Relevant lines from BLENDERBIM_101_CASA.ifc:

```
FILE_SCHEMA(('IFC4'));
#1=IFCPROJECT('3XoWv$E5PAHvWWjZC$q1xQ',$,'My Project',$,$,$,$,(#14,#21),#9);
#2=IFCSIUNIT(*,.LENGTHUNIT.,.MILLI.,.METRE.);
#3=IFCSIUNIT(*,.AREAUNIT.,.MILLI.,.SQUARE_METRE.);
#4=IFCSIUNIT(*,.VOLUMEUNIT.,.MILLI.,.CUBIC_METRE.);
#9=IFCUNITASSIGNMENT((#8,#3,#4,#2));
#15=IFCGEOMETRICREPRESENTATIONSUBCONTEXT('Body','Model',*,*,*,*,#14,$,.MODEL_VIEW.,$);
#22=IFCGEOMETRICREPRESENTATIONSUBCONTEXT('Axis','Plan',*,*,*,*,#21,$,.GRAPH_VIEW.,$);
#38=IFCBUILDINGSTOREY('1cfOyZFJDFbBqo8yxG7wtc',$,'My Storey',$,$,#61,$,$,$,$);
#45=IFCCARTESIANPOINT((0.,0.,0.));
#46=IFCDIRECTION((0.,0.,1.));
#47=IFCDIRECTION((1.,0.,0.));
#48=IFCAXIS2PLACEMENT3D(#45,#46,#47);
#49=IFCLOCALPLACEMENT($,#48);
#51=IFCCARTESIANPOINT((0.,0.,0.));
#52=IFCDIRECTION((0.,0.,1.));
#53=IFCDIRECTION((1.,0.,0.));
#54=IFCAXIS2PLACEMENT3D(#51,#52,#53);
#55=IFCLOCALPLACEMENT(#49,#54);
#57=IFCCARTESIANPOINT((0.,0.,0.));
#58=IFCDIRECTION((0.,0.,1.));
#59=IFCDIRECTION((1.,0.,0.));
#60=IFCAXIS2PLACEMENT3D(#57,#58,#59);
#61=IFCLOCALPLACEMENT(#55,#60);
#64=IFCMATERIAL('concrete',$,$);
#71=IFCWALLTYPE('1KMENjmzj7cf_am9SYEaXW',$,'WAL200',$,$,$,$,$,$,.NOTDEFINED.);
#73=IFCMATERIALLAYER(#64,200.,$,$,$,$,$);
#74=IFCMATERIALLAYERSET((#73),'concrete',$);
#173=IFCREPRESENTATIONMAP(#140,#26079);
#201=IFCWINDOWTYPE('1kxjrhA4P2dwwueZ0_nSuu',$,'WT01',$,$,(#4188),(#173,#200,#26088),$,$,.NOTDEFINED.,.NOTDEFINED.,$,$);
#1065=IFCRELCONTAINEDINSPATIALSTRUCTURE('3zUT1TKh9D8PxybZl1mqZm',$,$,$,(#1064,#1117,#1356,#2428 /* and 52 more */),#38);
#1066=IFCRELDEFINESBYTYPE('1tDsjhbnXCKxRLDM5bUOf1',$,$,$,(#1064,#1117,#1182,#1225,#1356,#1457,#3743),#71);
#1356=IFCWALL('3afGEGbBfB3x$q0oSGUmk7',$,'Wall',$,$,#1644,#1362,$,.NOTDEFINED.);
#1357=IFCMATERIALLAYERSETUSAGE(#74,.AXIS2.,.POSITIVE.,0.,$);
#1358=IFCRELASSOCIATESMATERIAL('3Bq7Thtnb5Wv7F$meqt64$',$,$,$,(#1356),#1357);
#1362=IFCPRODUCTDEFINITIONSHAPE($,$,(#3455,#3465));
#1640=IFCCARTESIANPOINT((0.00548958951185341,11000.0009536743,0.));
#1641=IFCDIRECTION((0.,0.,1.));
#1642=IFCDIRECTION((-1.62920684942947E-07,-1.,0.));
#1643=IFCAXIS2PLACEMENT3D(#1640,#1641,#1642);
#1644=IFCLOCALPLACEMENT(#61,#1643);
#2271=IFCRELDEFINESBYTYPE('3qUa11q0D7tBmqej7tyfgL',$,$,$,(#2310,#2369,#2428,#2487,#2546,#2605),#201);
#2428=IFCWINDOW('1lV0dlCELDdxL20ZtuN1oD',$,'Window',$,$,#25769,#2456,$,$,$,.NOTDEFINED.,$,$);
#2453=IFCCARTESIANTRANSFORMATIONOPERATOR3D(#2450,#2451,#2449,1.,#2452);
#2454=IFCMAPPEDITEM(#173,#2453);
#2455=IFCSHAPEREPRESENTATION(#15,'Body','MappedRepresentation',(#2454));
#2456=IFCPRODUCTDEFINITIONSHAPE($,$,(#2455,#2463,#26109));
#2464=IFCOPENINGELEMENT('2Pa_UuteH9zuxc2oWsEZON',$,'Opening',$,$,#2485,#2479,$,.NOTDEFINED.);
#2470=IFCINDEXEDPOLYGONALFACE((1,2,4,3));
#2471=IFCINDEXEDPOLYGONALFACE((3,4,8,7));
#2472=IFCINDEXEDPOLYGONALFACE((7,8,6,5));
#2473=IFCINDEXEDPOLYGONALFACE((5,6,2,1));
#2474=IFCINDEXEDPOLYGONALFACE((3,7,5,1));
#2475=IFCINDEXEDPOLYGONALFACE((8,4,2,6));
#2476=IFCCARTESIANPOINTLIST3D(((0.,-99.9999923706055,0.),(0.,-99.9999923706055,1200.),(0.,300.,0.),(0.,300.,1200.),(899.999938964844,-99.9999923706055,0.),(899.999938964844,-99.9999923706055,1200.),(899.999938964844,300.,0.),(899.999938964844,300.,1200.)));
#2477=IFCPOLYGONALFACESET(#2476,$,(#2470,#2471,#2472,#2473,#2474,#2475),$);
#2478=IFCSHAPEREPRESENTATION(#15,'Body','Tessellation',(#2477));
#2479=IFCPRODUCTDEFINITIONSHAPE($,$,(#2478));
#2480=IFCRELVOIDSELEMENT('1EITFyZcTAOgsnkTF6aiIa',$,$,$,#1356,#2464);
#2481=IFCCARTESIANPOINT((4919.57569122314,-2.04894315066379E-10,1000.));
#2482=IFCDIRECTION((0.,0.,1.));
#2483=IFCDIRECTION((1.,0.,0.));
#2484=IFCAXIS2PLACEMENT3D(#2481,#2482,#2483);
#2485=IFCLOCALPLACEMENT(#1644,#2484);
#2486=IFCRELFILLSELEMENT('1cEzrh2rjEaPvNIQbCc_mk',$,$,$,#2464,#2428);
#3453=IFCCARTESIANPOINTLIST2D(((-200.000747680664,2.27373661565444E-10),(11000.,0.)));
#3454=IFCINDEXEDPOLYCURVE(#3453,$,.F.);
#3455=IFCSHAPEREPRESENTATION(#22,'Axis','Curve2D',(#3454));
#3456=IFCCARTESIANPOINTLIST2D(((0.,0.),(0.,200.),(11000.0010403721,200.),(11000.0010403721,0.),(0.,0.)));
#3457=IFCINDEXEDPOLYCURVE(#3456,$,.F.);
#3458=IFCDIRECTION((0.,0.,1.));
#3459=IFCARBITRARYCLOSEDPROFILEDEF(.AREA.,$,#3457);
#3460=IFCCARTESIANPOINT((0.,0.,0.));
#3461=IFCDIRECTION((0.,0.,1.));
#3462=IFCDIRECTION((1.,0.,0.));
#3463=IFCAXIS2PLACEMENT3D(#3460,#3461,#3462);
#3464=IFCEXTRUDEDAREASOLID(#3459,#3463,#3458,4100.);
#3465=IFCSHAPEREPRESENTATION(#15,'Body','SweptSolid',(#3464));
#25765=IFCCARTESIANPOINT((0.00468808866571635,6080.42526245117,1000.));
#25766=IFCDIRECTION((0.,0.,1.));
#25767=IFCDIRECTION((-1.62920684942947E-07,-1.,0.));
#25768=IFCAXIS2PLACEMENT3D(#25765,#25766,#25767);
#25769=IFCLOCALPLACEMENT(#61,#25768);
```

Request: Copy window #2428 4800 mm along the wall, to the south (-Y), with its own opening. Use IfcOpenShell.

```python
import ifcopenshell
import ifcopenshell.api.feature
import ifcopenshell.api.geometry
import ifcopenshell.api.root
import ifcopenshell.geom
import ifcopenshell.util.element
import ifcopenshell.util.placement
import ifcopenshell.util.shape

model = ifcopenshell.open("BLENDERBIM_101_CASA.ifc")
settings = ifcopenshell.geom.settings()


def volume(element):
    """Net volume in cubic metres, openings subtracted."""
    shape = ifcopenshell.geom.create_shape(settings, element)
    return ifcopenshell.util.shape.get_volume(shape.geometry)


window = model.by_guid("1lV0dlCELDdxL20ZtuN1oD")
opening = window.FillsVoids[0].RelatingOpeningElement
wall = opening.VoidsElements[0].RelatingBuildingElement
before = volume(wall)
shift = ifcopenshell.util.placement.get_local_placement(wall.ObjectPlacement)[:3, 0] * 4800.0

# copy_class copies the void relationship, type, container and properties, but no geometry.
new_opening = ifcopenshell.api.root.copy_class(model, product=opening)
new_opening.Representation = ifcopenshell.util.element.copy_deep(
    model, opening.Representation, exclude=["IfcGeometricRepresentationContext", "IfcRepresentationMap"]
)
new_window = ifcopenshell.api.root.copy_class(model, product=window)
new_window.Representation = ifcopenshell.util.element.copy_deep(
    model, window.Representation, exclude=["IfcGeometricRepresentationContext", "IfcRepresentationMap"]
)
ifcopenshell.api.feature.add_filling(model, opening=new_opening, element=new_window)

for old, new in ((opening, new_opening), (window, new_window)):
    matrix = ifcopenshell.util.placement.get_local_placement(old.ObjectPlacement)
    matrix[:3, 3] += shift
    ifcopenshell.api.geometry.edit_object_placement(model, product=new, matrix=matrix, is_si=False)

after = volume(wall)

print(f"wall volume {before:.3f} -> {after:.3f} m3")

model.write("BLENDERBIM_101_CASA_v2.ifc")
```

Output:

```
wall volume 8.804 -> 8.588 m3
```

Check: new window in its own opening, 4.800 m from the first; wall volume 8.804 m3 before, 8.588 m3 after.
